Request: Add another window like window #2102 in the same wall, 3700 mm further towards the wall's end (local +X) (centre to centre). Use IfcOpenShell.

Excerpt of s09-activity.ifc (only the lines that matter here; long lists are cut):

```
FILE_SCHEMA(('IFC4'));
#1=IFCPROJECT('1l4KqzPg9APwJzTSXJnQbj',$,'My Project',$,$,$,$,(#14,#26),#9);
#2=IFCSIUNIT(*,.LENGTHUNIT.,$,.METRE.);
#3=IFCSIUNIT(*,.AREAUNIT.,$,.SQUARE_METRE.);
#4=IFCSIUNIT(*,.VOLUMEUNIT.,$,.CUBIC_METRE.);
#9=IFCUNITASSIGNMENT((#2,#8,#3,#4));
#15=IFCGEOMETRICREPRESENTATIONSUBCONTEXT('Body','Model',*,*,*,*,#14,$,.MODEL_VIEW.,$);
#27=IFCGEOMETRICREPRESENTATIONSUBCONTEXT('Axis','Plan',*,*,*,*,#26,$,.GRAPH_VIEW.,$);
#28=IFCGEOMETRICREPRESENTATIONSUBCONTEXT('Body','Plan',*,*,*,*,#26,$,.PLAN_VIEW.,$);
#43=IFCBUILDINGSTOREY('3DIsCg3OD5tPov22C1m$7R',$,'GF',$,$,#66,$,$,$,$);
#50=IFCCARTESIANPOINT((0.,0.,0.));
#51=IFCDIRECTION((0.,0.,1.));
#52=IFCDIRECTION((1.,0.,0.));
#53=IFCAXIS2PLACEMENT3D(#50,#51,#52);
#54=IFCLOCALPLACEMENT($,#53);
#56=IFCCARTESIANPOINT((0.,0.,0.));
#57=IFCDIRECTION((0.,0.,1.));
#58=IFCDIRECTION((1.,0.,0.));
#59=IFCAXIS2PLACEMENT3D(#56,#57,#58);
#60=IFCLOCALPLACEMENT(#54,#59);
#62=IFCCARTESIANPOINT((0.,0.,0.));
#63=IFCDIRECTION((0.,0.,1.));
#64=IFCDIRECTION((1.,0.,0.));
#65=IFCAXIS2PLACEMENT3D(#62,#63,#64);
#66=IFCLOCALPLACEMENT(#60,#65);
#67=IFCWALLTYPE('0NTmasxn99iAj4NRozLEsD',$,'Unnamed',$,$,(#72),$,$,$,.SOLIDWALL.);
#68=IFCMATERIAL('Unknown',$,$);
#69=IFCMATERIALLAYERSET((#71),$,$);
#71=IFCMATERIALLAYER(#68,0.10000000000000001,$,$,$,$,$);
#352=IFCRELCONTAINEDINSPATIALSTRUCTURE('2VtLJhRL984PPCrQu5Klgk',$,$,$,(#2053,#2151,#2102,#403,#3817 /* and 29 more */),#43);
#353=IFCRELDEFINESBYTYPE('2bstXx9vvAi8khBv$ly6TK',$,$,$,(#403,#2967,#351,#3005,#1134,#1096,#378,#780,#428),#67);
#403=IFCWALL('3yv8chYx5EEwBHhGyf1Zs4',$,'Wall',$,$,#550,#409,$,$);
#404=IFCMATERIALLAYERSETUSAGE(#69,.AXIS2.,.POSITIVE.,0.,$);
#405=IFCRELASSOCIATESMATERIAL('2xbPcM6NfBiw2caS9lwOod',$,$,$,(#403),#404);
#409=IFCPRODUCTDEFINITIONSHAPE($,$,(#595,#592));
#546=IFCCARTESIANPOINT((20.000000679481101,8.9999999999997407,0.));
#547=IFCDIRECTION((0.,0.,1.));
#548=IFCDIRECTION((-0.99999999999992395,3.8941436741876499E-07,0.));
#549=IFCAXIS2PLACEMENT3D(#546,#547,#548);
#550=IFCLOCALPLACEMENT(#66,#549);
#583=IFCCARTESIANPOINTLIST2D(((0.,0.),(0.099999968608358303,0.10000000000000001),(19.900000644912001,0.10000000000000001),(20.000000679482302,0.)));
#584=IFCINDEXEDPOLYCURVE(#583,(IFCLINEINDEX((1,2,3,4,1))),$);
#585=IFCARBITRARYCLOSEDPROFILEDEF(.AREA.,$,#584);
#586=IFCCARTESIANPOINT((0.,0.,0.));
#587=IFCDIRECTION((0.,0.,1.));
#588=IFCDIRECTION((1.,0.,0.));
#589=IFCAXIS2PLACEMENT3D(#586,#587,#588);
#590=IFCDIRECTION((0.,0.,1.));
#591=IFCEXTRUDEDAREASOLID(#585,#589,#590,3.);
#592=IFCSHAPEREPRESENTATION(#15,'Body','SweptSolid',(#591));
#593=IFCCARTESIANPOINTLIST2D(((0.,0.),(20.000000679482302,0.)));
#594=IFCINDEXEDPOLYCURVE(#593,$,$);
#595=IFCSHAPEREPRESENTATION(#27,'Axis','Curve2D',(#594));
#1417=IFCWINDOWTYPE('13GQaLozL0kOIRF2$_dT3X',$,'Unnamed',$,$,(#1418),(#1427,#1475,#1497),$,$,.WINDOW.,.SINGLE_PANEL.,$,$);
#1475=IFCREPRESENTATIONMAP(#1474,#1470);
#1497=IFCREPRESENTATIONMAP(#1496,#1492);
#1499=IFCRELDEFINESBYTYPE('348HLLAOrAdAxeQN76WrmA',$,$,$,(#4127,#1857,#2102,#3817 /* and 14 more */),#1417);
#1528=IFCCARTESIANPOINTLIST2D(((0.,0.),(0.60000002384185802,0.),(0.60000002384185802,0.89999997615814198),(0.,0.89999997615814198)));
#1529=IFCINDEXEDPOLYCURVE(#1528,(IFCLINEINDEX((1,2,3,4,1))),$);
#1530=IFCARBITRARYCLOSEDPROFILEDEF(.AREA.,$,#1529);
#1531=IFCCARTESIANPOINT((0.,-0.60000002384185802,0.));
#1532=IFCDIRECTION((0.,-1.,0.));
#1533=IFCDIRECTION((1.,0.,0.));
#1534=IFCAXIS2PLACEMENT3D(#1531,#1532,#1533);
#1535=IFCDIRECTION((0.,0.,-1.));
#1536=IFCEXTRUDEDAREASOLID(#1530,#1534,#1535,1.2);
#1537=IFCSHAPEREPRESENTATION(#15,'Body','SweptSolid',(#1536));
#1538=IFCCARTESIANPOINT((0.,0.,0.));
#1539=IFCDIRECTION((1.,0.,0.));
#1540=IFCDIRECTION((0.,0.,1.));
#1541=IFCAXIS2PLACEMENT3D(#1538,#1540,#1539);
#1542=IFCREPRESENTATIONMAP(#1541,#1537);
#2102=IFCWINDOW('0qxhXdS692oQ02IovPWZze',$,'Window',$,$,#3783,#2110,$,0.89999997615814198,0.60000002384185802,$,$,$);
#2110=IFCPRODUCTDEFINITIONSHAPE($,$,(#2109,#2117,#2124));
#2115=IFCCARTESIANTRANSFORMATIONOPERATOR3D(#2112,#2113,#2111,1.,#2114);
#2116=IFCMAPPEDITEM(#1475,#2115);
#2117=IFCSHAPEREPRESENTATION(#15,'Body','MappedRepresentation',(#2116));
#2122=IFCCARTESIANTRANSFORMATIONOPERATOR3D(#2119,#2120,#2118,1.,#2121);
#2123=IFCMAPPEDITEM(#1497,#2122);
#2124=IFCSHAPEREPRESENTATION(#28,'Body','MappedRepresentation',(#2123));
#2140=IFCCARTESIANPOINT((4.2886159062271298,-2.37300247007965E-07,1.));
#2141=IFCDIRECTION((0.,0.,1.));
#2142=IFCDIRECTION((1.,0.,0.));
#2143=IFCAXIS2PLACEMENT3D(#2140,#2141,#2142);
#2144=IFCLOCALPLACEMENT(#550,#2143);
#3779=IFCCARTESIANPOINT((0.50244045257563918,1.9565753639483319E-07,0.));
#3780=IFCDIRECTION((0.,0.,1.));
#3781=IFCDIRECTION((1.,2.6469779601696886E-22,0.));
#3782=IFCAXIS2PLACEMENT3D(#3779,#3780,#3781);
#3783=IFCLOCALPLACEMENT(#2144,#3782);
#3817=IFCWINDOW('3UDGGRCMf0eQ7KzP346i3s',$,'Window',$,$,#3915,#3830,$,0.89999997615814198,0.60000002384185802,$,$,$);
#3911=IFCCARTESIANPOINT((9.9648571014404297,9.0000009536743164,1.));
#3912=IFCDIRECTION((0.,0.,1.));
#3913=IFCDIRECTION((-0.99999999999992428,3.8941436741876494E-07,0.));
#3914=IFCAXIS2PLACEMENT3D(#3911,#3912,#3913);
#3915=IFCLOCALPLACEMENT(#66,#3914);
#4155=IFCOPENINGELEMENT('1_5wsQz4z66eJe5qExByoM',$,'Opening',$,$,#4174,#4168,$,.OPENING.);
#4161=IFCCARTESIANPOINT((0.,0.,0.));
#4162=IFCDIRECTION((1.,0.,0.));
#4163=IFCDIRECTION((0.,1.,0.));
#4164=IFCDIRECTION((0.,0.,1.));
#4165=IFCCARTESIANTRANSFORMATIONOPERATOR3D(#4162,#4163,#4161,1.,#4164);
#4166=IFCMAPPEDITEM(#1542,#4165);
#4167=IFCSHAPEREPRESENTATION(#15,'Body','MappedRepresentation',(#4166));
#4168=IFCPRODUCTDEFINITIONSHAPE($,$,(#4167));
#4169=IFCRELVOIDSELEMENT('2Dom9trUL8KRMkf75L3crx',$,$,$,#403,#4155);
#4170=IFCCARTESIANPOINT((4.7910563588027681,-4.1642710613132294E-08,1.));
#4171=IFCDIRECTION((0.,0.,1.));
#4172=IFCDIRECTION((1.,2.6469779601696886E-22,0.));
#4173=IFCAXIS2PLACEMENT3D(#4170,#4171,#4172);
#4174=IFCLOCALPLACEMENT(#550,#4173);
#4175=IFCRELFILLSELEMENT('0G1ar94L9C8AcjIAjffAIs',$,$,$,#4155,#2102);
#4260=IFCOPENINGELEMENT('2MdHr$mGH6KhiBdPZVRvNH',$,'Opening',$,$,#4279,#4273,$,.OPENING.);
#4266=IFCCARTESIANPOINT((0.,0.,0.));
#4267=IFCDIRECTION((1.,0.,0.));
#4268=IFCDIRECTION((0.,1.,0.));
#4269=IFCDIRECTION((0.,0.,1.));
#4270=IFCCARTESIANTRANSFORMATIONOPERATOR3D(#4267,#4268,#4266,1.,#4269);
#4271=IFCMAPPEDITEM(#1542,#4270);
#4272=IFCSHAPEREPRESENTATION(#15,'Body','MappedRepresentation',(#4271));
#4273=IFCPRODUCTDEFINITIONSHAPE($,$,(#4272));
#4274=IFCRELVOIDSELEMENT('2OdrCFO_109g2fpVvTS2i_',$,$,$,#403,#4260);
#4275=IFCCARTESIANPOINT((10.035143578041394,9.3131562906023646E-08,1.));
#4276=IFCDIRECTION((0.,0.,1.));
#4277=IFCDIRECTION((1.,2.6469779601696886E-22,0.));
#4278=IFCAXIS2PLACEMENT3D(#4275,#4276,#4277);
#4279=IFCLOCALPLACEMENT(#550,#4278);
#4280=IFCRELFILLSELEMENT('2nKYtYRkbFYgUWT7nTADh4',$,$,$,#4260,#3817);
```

```python
import ifcopenshell
import ifcopenshell.api.feature
import ifcopenshell.api.geometry
import ifcopenshell.api.root
import ifcopenshell.geom
import ifcopenshell.util.element
import ifcopenshell.util.placement
import ifcopenshell.util.shape
import ifcopenshell.util.unit

model = ifcopenshell.open("s09-activity.ifc")
unit_scale = ifcopenshell.util.unit.calculate_unit_scale(model)
settings = ifcopenshell.geom.settings()


def volume(element):
    """Net volume in cubic metres, openings subtracted."""
    shape = ifcopenshell.geom.create_shape(settings, element)
    return ifcopenshell.util.shape.get_volume(shape.geometry)


window = model.by_guid("0qxhXdS692oQ02IovPWZze")
opening = window.FillsVoids[0].RelatingOpeningElement
wall = opening.VoidsElements[0].RelatingBuildingElement
before = volume(wall)
shift = ifcopenshell.util.placement.get_local_placement(wall.ObjectPlacement)[:3, 0] * 3.7 / unit_scale

# copy_class copies the void relationship, type, container and properties, but no geometry.
new_opening = ifcopenshell.api.root.copy_class(model, product=opening)
new_opening.Representation = ifcopenshell.util.element.copy_deep(
    model, opening.Representation, exclude=["IfcGeometricRepresentationContext", "IfcRepresentationMap"]
)
new_window = ifcopenshell.api.root.copy_class(model, product=window)
new_window.Representation = ifcopenshell.util.element.copy_deep(
    model, window.Representation, exclude=["IfcGeometricRepresentationContext", "IfcRepresentationMap"]
)
ifcopenshell.api.feature.add_filling(model, opening=new_opening, element=new_window)

for old, new in ((opening, new_opening), (window, new_window)):
    matrix = ifcopenshell.util.placement.get_local_placement(old.ObjectPlacement)
    matrix[:3, 3] += shift
    ifcopenshell.api.geometry.edit_object_placement(model, product=new, matrix=matrix, is_si=False)

after = volume(wall)

print(f"wall volume {before:.3f} -> {after:.3f} m3")

model.write("s09-activity_edited.ifc")
```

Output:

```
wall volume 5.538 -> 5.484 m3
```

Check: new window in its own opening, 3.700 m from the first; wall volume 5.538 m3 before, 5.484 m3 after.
